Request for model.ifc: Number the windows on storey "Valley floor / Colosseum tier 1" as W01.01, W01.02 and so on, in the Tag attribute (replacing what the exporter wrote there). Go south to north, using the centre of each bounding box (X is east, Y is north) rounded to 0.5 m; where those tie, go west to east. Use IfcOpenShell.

First a look at what the model holds.

```python
import ifcopenshell
import ifcopenshell.util.element
import ifcopenshell.util.placement

model = ifcopenshell.open("model.ifc")
print(model.schema)
storey = next(s for s in model.by_type("IfcBuildingStorey") if s.Name == "Valley floor / Colosseum tier 1")
windows = [e for e in ifcopenshell.util.element.get_decomposition(storey) if e.is_a("IfcWindow")]
for e in sorted(windows, key=lambda e: e.id()):
    origin = ifcopenshell.util.placement.get_local_placement(e.ObjectPlacement)[:3, 3]
    print(e.id(), e.Tag, e.Name, origin.round(2) + 0.0, sep=" | ")
```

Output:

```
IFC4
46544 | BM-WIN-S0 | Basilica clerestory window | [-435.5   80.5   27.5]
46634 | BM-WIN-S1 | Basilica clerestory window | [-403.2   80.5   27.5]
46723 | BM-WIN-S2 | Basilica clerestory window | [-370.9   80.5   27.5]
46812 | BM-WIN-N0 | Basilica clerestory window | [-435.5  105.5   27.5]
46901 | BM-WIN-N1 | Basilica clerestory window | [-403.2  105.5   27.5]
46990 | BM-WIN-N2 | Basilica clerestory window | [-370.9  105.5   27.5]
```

```python
import ifcopenshell
import ifcopenshell.geom
import ifcopenshell.util.element
import ifcopenshell.util.shape

model = ifcopenshell.open("model.ifc")
settings = ifcopenshell.geom.settings()
settings.set("use-world-coords", True)


def centre(element):
    shape = ifcopenshell.geom.create_shape(settings, element)
    return ifcopenshell.util.shape.get_bbox_centroid(shape.geometry)


storey = next(s for s in model.by_type("IfcBuildingStorey") if s.Name == "Valley floor / Colosseum tier 1")
windows = [e for e in ifcopenshell.util.element.get_decomposition(storey) if e.is_a("IfcWindow")]

# Insertion points can sit at a corner or the storey origin, so sort by the geometry (in metres).
centres = {e: centre(e) for e in windows}
windows.sort(key=lambda e: (round(centres[e][1] / 0.5), centres[e][0]))

for i, e in enumerate(windows, start=1):
    number = f"W01.{i:02d}"
    e.Tag = number
    print(e.id(), number)

model.write("model_v2.ifc")
```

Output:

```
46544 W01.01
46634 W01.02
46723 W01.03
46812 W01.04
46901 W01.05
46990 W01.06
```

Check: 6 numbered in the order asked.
